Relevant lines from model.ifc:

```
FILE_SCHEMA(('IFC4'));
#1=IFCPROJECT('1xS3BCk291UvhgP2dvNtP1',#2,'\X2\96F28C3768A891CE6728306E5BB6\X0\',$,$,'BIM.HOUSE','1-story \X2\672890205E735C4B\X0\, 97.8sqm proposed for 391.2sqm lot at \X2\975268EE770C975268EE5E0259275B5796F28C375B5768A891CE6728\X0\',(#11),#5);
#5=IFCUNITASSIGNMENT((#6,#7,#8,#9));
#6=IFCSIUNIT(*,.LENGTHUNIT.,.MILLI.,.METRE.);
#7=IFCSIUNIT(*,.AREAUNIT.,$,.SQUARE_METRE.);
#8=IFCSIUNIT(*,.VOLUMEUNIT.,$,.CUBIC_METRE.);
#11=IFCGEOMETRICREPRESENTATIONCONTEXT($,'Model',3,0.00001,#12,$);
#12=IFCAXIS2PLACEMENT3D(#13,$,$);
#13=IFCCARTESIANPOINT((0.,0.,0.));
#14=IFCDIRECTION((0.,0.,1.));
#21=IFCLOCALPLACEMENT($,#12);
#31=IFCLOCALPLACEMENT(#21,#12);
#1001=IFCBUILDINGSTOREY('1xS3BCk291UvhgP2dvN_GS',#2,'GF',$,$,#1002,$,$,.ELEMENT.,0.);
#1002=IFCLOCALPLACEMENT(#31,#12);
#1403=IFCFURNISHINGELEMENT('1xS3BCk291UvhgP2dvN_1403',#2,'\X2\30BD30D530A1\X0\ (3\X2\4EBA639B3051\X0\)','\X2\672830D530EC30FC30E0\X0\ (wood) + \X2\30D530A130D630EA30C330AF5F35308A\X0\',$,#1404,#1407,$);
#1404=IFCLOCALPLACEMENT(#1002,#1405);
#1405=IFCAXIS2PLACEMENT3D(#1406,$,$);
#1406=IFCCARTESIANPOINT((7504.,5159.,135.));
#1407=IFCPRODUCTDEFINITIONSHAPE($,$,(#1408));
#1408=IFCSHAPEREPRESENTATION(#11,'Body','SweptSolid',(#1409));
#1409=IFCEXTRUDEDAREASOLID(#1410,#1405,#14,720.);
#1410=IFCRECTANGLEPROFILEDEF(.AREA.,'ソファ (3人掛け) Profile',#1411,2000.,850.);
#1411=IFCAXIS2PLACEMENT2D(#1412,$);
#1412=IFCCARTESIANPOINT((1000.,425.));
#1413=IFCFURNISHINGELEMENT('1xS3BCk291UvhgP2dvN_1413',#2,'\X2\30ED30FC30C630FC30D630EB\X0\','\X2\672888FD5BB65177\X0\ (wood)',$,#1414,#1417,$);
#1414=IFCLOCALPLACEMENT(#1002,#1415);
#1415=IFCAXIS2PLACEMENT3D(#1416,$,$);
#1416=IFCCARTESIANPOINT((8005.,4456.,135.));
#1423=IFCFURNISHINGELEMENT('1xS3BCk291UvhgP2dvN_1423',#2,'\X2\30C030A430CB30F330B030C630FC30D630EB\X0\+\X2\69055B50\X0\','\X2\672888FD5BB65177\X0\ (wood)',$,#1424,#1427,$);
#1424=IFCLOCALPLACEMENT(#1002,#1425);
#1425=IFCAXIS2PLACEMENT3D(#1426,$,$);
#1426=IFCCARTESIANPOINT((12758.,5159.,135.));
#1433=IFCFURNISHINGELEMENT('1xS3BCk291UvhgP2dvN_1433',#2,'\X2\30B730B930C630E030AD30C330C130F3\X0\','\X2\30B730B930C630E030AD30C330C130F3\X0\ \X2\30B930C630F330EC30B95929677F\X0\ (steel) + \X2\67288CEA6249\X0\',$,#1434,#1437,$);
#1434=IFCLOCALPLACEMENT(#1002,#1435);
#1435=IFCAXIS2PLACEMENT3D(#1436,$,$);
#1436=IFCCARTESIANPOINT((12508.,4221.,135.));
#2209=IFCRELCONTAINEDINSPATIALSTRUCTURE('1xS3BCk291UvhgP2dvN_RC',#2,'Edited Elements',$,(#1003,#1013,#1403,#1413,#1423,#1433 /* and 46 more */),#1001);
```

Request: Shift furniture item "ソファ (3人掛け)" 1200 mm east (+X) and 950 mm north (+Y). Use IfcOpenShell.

```python
import ifcopenshell
import ifcopenshell.api.geometry
import ifcopenshell.util.placement

model = ifcopenshell.open("model.ifc")

item = model.by_guid("1xS3BCk291UvhgP2dvN_1403")
matrix = ifcopenshell.util.placement.get_local_placement(item.ObjectPlacement)
matrix[0, 3] += 1200.0
matrix[1, 3] += 950.0
ifcopenshell.api.geometry.edit_object_placement(model, product=item, matrix=matrix, is_si=False)

print(ifcopenshell.util.placement.get_local_placement(item.ObjectPlacement).round(3) + 0.0)

model.write("model_edited.ifc")
```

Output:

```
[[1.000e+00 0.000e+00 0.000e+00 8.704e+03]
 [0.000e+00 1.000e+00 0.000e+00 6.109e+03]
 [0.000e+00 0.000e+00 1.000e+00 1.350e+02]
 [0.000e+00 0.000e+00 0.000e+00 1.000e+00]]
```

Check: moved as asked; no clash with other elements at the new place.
